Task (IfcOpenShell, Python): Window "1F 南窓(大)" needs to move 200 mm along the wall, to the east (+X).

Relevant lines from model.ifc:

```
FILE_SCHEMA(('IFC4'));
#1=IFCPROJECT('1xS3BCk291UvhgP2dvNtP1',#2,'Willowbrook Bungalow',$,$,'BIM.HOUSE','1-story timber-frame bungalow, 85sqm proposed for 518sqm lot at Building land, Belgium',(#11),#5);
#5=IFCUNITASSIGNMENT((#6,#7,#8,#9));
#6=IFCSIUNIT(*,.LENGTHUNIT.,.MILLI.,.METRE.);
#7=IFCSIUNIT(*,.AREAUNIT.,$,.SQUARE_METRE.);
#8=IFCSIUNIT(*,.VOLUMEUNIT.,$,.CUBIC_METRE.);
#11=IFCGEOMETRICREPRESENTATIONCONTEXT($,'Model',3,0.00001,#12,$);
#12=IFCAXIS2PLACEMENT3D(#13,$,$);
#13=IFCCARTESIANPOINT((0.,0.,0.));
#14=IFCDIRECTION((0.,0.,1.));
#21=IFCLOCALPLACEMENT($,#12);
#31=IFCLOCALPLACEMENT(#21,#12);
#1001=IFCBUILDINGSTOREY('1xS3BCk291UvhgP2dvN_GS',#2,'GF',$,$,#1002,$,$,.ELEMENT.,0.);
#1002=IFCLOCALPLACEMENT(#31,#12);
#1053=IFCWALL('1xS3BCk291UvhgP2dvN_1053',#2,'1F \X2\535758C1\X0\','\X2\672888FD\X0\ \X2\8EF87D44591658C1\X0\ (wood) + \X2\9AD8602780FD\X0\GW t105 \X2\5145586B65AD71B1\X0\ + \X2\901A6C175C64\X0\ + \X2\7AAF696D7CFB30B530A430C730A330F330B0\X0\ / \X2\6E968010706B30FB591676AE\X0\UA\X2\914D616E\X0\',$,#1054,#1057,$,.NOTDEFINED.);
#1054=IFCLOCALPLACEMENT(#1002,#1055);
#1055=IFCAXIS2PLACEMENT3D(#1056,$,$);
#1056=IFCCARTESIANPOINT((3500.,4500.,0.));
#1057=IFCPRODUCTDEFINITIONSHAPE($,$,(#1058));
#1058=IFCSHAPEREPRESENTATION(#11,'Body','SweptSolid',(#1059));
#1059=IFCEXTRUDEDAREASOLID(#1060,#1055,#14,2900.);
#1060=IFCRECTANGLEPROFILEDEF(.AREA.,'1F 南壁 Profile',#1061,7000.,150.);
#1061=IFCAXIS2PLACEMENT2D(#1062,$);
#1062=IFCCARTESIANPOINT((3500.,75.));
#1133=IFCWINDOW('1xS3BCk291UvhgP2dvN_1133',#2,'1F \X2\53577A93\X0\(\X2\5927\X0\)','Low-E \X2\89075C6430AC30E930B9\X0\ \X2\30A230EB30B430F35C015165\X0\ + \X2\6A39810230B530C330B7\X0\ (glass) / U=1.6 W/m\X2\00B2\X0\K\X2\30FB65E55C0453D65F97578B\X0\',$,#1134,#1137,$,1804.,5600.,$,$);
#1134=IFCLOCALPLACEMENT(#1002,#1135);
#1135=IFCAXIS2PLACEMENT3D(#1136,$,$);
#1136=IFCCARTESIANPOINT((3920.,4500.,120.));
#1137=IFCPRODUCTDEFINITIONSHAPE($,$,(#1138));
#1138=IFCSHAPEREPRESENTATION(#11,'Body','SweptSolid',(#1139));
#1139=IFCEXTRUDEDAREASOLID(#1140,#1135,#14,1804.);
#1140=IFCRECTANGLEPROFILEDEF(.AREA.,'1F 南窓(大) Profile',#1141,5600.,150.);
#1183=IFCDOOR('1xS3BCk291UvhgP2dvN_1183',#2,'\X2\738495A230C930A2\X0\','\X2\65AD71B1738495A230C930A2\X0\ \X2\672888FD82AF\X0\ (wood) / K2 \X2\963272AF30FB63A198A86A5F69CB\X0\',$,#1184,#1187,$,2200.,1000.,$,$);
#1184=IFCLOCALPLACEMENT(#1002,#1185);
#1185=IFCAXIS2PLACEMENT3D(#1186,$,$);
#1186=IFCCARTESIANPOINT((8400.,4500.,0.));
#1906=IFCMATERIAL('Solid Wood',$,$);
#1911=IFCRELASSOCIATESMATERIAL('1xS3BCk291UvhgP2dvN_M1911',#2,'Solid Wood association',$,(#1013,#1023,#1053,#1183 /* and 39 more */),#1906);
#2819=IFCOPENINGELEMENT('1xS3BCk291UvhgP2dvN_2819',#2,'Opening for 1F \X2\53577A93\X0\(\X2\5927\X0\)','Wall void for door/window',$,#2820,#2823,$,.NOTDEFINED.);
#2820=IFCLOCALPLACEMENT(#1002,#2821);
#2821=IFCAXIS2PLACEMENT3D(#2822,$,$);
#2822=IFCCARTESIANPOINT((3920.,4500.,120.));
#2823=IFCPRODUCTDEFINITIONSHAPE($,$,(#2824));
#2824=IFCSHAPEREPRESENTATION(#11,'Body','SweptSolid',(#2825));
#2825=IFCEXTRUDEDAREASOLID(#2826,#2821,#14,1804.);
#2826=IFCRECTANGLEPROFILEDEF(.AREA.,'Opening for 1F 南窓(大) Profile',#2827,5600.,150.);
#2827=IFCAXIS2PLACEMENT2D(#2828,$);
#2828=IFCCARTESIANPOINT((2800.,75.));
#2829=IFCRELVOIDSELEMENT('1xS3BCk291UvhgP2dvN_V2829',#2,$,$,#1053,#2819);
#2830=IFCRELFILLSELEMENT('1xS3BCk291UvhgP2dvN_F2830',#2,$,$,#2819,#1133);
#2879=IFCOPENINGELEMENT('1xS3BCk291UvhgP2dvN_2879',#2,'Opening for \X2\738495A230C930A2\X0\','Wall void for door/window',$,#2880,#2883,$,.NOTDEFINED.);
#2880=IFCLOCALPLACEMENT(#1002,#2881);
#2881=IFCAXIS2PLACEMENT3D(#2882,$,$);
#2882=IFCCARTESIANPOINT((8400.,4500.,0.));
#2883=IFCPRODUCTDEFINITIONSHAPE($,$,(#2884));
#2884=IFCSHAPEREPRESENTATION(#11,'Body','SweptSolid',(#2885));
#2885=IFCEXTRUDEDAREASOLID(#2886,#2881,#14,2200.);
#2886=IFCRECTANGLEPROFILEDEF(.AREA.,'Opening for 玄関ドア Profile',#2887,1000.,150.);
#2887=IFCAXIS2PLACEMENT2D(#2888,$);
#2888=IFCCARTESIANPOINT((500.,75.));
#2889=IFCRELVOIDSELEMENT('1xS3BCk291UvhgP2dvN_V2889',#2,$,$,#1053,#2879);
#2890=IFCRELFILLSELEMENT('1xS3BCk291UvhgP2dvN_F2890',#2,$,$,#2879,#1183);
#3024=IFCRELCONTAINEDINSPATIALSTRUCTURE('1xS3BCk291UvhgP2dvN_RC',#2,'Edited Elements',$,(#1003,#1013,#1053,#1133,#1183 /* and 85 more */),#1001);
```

```python
import ifcopenshell
import ifcopenshell.api.geometry
import ifcopenshell.util.placement

model = ifcopenshell.open("model.ifc")

window = model.by_guid("1xS3BCk291UvhgP2dvN_1133")
opening = window.FillsVoids[0].RelatingOpeningElement
wall = opening.VoidsElements[0].RelatingBuildingElement

wall_matrix = ifcopenshell.util.placement.get_local_placement(wall.ObjectPlacement)
shift = wall_matrix[:3, 0] * 200.0
before = ifcopenshell.util.placement.get_local_placement(window.ObjectPlacement)[:3, 3].copy()

# The window is not placed relative to its opening, so move both.
for product in (opening, window):
    matrix = ifcopenshell.util.placement.get_local_placement(product.ObjectPlacement)
    matrix[:3, 3] += shift
    ifcopenshell.api.geometry.edit_object_placement(model, product=product, matrix=matrix, is_si=False)

after = ifcopenshell.util.placement.get_local_placement(window.ObjectPlacement)[:3, 3]
print("window moved by", (after - before).round(3) + 0.0)

model.write("model_rev.ifc")
```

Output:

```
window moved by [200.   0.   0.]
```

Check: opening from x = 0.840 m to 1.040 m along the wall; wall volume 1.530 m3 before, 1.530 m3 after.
